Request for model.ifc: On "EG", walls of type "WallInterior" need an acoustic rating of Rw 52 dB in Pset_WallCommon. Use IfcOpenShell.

First a look at what the model holds.

```python
import ifcopenshell
import ifcopenshell.util.element

model = ifcopenshell.open("model.ifc")
print(model.schema)
storey = next(s for s in model.by_type("IfcBuildingStorey") if s.Name == "EG")
walls = [e for e in ifcopenshell.util.element.get_decomposition(storey) if e.is_a("IfcWall")]
seen = {}
for e in walls:
    element_type = ifcopenshell.util.element.get_type(e)
    key = (element_type.Name if element_type != e and element_type else None, ifcopenshell.util.element.get_pset(e, "Pset_WallCommon", "AcousticRating"))
    seen[key] = seen.get(key, 0) + 1
for (name, value), count in sorted(seen.items(), key=str):
    print(count, "x", name, "|", value)
```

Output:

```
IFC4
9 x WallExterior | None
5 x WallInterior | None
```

```python
import ifcopenshell
import ifcopenshell.api.pset
import ifcopenshell.util.element

model = ifcopenshell.open("model.ifc")

storey = next(s for s in model.by_type("IfcBuildingStorey") if s.Name == "EG")
walls = [e for e in ifcopenshell.util.element.get_decomposition(storey) if e.is_a("IfcWall")]

count = 0
for e in walls:
    element_type = ifcopenshell.util.element.get_type(e)
    if element_type in (None, e) or element_type.Name != "WallInterior":
        continue
    # add_pset returns the element's existing set when there is one.
    pset = ifcopenshell.api.pset.add_pset(model, product=e, name="Pset_WallCommon")
    ifcopenshell.api.pset.edit_pset(model, pset=pset, properties={"AcousticRating": "Rw 52 dB"})
    count += 1

print(count, "walls updated")

model.write("model_edited.ifc")
```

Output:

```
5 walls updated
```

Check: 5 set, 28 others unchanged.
